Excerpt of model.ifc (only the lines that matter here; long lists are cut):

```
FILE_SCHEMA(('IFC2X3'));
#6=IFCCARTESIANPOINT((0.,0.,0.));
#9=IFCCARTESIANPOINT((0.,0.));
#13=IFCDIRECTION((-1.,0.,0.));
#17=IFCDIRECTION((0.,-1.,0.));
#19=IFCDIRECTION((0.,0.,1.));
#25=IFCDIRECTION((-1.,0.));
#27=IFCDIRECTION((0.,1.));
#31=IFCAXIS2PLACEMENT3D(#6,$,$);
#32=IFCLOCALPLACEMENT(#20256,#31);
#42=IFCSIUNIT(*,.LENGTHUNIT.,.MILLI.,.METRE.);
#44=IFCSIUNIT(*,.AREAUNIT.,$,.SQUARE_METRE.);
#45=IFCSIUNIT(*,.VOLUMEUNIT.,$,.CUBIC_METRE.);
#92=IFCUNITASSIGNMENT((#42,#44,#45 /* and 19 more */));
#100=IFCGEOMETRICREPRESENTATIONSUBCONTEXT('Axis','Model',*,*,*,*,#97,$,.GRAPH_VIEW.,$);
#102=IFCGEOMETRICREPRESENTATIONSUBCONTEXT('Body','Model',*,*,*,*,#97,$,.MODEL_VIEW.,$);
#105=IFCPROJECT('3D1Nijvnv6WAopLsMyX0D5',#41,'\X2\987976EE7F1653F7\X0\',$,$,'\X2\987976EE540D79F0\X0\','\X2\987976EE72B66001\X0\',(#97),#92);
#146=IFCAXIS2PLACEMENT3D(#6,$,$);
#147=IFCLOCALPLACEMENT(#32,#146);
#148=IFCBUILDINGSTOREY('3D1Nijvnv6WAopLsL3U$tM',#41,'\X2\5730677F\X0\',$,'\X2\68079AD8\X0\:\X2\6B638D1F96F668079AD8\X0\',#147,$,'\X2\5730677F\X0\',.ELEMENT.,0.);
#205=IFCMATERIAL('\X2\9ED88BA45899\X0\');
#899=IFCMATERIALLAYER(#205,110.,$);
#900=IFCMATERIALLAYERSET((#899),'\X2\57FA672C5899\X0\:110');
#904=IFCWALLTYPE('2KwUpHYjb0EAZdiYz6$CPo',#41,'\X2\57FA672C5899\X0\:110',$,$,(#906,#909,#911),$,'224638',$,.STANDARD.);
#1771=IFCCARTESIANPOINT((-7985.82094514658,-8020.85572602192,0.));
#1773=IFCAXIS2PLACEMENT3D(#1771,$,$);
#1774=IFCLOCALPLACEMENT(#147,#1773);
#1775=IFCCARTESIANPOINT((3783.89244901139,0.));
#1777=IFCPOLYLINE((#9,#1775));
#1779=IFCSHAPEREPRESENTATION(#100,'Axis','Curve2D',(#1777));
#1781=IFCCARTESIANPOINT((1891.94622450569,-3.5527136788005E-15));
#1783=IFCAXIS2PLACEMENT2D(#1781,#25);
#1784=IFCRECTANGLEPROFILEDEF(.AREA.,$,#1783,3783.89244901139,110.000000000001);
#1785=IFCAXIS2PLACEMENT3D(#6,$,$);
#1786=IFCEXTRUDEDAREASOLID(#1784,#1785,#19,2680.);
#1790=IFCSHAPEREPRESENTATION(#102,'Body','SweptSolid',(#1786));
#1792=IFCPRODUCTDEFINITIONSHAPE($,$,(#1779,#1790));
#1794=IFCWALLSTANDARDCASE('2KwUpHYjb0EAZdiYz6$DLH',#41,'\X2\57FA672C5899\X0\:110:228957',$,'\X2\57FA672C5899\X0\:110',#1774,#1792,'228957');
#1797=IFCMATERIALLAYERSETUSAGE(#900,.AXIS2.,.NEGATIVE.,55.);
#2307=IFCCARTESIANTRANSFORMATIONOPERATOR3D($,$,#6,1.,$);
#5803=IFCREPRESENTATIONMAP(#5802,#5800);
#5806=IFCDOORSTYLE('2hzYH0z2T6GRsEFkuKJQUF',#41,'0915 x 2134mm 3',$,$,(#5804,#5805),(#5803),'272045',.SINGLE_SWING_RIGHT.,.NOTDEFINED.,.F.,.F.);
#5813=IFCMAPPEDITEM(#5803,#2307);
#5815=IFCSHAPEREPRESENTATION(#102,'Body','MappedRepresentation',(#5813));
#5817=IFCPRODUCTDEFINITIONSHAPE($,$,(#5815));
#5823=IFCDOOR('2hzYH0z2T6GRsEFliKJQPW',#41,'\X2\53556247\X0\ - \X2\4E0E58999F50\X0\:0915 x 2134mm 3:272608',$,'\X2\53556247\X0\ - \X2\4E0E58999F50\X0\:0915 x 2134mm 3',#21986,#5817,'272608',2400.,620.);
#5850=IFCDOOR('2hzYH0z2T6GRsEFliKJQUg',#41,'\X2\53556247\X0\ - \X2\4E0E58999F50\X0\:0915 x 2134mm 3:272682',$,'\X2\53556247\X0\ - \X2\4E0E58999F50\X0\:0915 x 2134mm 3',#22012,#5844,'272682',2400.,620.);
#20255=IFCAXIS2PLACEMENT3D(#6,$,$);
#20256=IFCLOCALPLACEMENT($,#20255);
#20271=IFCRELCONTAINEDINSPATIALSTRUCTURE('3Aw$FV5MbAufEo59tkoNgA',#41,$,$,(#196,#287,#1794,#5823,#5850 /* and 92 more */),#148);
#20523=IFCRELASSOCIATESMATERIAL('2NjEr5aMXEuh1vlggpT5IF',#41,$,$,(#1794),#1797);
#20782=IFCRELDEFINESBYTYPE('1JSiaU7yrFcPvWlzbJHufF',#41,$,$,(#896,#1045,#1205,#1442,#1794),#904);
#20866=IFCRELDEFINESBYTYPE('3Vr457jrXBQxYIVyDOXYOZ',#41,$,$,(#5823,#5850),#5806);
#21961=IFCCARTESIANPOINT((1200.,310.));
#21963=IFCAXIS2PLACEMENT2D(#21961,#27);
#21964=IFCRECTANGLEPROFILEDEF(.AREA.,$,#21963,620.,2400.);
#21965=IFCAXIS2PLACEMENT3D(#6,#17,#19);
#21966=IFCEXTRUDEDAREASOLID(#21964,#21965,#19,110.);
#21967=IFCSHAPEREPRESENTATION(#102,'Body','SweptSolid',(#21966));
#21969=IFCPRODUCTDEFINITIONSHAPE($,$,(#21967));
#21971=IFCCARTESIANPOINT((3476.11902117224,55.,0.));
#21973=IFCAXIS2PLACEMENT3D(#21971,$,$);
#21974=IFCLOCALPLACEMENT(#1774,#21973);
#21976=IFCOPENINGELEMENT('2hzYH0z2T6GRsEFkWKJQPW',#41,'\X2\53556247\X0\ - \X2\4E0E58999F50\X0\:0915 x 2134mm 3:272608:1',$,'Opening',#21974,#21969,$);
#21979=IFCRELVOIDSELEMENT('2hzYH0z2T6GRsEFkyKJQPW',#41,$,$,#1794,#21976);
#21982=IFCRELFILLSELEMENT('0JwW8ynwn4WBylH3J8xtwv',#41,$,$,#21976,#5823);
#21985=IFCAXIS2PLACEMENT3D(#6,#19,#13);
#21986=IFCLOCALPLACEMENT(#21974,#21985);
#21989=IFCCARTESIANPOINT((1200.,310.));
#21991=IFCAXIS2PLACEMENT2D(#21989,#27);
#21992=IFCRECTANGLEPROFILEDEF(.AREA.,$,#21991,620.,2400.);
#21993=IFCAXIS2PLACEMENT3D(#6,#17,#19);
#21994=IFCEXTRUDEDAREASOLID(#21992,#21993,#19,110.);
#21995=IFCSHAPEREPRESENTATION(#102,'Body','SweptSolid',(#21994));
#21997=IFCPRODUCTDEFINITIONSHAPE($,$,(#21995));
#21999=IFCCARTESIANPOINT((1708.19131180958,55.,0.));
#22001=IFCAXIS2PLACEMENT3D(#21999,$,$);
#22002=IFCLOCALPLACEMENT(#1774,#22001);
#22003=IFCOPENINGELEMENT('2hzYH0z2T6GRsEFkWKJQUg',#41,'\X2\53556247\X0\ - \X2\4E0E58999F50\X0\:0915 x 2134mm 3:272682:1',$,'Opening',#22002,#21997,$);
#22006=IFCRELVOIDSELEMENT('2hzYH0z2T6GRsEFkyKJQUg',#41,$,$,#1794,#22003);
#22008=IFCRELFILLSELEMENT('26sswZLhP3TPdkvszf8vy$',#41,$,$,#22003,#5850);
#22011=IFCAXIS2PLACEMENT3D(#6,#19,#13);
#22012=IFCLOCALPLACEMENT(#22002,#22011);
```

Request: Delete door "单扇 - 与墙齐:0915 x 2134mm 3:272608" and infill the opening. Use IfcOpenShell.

```python
import ifcopenshell
import ifcopenshell.api.feature
import ifcopenshell.api.root
import ifcopenshell.geom
import ifcopenshell.util.shape

model = ifcopenshell.open("model.ifc")
settings = ifcopenshell.geom.settings()


def volume(element):
    """Net volume in cubic metres, openings subtracted."""
    shape = ifcopenshell.geom.create_shape(settings, element)
    return ifcopenshell.util.shape.get_volume(shape.geometry)


door = model.by_guid("2hzYH0z2T6GRsEFliKJQPW")
opening = door.FillsVoids[0].RelatingOpeningElement
wall = opening.VoidsElements[0].RelatingBuildingElement
before = volume(wall)

ifcopenshell.api.root.remove_product(model, product=door)
ifcopenshell.api.feature.remove_feature(model, feature=opening)

after = volume(wall)

print(f"wall volume {before:.3f} -> {after:.3f} m3")

model.write("model-out.ifc")
```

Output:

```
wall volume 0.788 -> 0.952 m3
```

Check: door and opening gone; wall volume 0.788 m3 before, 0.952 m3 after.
